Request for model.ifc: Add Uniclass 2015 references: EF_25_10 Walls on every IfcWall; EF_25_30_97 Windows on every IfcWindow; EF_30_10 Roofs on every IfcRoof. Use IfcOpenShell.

First a look at what the model holds.

```python
import ifcopenshell

model = ifcopenshell.open("model.ifc")
print(model.schema)
print("classifications:", [c.Name for c in model.by_type("IfcClassification")])
for ifc_class in ("IfcDoor", "IfcRoof", "IfcStair", "IfcWall", "IfcWindow"):
    print(ifc_class, len(model.by_type(ifc_class)))
```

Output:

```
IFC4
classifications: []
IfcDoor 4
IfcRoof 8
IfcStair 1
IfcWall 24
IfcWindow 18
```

```python
import ifcopenshell
import ifcopenshell.api.classification

model = ifcopenshell.open("model.ifc")

system = ifcopenshell.api.classification.add_classification(model, classification="Uniclass 2015")

codes = {
    "IfcWall": ("EF_25_10", "Walls"),
    "IfcWindow": ("EF_25_30_97", "Windows"),
    "IfcRoof": ("EF_30_10", "Roofs"),
}
for ifc_class, (code, name) in codes.items():
    products = model.by_type(ifc_class)
    ifcopenshell.api.classification.add_reference(
        model, products=products, classification=system, identification=code, name=name
    )
    print(code, len(products))

model.write("model_edited.ifc")
```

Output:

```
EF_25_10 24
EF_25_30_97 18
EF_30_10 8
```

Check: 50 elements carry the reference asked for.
